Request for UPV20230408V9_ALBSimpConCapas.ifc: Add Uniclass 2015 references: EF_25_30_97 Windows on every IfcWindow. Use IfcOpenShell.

First a look at what the model holds.

```python
import ifcopenshell

model = ifcopenshell.open("UPV20230408V9_ALBSimpConCapas.ifc")
print(model.schema)
print("classifications:", [c.Name for c in model.by_type("IfcClassification")])
for ifc_class in ("IfcDoor", "IfcRoof", "IfcStair", "IfcWall", "IfcWindow"):
    print(ifc_class, len(model.by_type(ifc_class)))
```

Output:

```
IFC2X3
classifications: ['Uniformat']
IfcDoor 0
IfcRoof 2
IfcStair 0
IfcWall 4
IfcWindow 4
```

```python
import ifcopenshell
import ifcopenshell.api.classification

model = ifcopenshell.open("UPV20230408V9_ALBSimpConCapas.ifc")

# IFC2X3 requires Source and Edition and has no link from the project to the system.
system = model.create_entity("IfcClassification", Source="NBS", Edition="2015", Name="Uniclass 2015")

codes = {
    "IfcWindow": ("EF_25_30_97", "Windows"),
}
for ifc_class, (code, name) in codes.items():
    products = model.by_type(ifc_class)
    ifcopenshell.api.classification.add_reference(
        model, products=products, classification=system, identification=code, name=name
    )
    print(code, len(products))

model.write("UPV20230408V9_ALBSimpConCapas_rev.ifc")
```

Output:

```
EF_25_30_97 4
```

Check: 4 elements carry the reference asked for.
